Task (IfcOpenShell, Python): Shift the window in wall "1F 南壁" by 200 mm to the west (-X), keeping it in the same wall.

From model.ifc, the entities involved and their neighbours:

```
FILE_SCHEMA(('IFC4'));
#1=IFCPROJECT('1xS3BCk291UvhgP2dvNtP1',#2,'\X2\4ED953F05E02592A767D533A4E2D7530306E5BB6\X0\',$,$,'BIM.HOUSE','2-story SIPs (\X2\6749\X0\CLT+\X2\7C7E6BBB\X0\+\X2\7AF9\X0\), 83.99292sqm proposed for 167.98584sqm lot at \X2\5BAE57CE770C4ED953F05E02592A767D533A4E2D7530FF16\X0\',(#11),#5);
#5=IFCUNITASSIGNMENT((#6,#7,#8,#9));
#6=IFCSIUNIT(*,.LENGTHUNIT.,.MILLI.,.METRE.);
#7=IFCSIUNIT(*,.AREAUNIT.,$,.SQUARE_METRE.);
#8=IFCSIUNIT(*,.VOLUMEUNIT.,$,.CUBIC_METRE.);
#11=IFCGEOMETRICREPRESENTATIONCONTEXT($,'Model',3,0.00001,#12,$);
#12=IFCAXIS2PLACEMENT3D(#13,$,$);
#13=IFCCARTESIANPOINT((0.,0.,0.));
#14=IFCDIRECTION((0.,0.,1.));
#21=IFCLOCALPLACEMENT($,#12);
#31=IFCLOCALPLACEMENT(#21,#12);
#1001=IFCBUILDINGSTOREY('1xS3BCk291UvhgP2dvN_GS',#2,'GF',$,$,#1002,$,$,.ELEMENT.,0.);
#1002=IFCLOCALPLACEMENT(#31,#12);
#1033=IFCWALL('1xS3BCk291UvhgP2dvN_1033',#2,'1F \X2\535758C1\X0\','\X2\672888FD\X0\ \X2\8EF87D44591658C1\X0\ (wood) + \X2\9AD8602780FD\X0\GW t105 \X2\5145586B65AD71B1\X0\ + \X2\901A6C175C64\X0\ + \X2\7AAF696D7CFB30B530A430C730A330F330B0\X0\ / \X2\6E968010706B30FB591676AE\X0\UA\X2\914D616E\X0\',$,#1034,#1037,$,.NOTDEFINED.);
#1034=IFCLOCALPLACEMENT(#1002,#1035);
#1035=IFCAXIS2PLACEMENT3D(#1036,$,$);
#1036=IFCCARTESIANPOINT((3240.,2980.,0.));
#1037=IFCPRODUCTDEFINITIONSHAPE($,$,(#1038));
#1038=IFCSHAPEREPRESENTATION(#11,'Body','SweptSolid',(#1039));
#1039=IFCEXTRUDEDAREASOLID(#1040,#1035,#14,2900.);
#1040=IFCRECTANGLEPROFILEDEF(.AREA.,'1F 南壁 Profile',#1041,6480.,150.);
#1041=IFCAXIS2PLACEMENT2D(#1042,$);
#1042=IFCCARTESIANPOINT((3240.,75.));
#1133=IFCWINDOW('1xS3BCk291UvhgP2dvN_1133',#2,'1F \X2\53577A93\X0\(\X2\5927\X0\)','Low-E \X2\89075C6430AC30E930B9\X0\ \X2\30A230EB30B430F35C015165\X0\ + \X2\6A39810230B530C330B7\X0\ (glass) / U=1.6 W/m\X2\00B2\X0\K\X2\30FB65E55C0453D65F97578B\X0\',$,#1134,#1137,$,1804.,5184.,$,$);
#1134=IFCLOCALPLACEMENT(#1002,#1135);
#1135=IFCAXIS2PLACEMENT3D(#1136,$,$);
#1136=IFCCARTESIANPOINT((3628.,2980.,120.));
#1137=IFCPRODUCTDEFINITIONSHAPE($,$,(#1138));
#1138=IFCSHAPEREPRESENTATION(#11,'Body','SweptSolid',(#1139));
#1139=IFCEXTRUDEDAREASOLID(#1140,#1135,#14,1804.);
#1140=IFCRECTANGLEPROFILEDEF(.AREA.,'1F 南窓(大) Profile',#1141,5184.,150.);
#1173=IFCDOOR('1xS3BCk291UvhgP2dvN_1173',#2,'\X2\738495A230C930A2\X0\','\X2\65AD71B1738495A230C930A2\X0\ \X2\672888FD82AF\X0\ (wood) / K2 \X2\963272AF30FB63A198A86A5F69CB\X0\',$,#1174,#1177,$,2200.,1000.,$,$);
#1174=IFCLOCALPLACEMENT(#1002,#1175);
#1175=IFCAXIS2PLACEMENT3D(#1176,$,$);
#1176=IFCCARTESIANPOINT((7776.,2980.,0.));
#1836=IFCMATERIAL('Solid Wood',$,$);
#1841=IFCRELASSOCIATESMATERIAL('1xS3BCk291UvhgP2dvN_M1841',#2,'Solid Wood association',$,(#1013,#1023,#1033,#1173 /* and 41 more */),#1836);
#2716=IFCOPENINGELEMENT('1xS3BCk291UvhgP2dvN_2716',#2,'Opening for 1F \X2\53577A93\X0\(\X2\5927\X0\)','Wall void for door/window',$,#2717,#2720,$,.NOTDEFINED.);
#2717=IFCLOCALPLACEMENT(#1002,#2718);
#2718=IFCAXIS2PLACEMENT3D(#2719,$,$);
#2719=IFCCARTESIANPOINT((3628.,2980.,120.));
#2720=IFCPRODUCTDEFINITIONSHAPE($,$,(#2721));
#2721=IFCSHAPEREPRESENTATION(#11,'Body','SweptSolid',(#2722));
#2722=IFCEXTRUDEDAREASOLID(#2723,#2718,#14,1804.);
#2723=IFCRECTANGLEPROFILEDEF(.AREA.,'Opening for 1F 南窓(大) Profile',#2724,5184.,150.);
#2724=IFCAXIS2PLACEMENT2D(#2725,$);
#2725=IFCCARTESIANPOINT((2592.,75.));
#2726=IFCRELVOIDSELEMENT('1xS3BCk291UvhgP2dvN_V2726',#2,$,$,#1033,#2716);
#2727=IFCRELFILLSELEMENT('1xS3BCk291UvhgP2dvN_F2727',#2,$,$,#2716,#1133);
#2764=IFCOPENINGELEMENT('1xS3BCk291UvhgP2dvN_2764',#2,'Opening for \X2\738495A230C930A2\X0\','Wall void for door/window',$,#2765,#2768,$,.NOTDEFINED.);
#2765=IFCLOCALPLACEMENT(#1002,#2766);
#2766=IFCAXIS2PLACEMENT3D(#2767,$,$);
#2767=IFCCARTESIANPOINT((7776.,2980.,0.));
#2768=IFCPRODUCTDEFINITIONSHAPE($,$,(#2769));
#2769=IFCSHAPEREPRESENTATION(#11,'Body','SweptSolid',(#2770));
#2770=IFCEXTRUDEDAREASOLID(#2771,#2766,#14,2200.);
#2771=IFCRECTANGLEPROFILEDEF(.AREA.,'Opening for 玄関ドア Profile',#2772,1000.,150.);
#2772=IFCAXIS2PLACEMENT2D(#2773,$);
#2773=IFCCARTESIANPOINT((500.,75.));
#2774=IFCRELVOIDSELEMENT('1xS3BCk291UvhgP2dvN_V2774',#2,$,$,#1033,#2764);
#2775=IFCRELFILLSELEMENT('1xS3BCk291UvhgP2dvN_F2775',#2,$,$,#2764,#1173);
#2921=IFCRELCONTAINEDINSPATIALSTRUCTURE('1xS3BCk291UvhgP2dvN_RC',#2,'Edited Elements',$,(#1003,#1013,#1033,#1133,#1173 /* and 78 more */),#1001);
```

```python
import ifcopenshell
import ifcopenshell.api.geometry
import ifcopenshell.util.placement
import ifcopenshell.util.unit

model = ifcopenshell.open("model.ifc")
unit_scale = ifcopenshell.util.unit.calculate_unit_scale(model)

window = model.by_guid("1xS3BCk291UvhgP2dvN_1133")
opening = window.FillsVoids[0].RelatingOpeningElement
wall = opening.VoidsElements[0].RelatingBuildingElement

wall_matrix = ifcopenshell.util.placement.get_local_placement(wall.ObjectPlacement)
shift = wall_matrix[:3, 0] * -0.2 / unit_scale
before = ifcopenshell.util.placement.get_local_placement(window.ObjectPlacement)[:3, 3].copy()

# The window is not placed relative to its opening, so move both.
for product in (opening, window):
    matrix = ifcopenshell.util.placement.get_local_placement(product.ObjectPlacement)
    matrix[:3, 3] += shift
    ifcopenshell.api.geometry.edit_object_placement(model, product=product, matrix=matrix, is_si=False)

after = ifcopenshell.util.placement.get_local_placement(window.ObjectPlacement)[:3, 3]
print("window moved by", (after - before).round(3) + 0.0)

model.write("model_rev.ifc")
```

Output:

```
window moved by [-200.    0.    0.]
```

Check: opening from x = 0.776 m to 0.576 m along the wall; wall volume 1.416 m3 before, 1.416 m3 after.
